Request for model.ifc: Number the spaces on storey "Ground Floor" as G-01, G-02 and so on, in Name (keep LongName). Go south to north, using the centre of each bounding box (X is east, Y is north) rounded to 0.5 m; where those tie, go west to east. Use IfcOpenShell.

First a look at what the model holds.

```python
import ifcopenshell
import ifcopenshell.util.element
import ifcopenshell.util.placement

model = ifcopenshell.open("model.ifc")
print(model.schema)
storey = next(s for s in model.by_type("IfcBuildingStorey") if s.Name == "Ground Floor")
spaces = [e for e in ifcopenshell.util.element.get_decomposition(storey) if e.is_a("IfcSpace")]
for e in sorted(spaces, key=lambda e: e.id()):
    origin = ifcopenshell.util.placement.get_local_placement(e.ObjectPlacement)[:3, 3]
    print(e.id(), e.Name, e.LongName, origin.round(2) + 0.0, sep=" | ")
```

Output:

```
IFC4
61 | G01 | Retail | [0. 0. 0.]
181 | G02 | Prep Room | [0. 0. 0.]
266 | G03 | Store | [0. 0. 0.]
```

```python
import ifcopenshell
import ifcopenshell.geom
import ifcopenshell.util.element
import ifcopenshell.util.shape

model = ifcopenshell.open("model.ifc")
settings = ifcopenshell.geom.settings()
settings.set("use-world-coords", True)


def centre(element):
    shape = ifcopenshell.geom.create_shape(settings, element)
    return ifcopenshell.util.shape.get_bbox_centroid(shape.geometry)


storey = next(s for s in model.by_type("IfcBuildingStorey") if s.Name == "Ground Floor")
spaces = [e for e in ifcopenshell.util.element.get_decomposition(storey) if e.is_a("IfcSpace")]

# Insertion points can sit at a corner or the storey origin, so sort by the geometry (in metres).
centres = {e: centre(e) for e in spaces}
spaces.sort(key=lambda e: (round(centres[e][1] / 0.5), centres[e][0]))

for i, e in enumerate(spaces, start=1):
    number = f"G-{i:02d}"
    e.Name = number
    print(e.id(), number)

model.write("model_v2.ifc")
```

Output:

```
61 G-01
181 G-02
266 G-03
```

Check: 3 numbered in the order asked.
